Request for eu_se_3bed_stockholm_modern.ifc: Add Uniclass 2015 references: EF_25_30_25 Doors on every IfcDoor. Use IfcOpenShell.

First a look at what the model holds.

```python
import ifcopenshell

model = ifcopenshell.open("eu_se_3bed_stockholm_modern.ifc")
print(model.schema)
print("classifications:", [c.Name for c in model.by_type("IfcClassification")])
for ifc_class in ("IfcDoor", "IfcRoof", "IfcStair", "IfcWall", "IfcWindow"):
    print(ifc_class, len(model.by_type(ifc_class)))
```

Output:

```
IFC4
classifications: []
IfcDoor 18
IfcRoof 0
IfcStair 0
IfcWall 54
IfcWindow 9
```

```python
import ifcopenshell
import ifcopenshell.api.classification

model = ifcopenshell.open("eu_se_3bed_stockholm_modern.ifc")

system = ifcopenshell.api.classification.add_classification(model, classification="Uniclass 2015")

codes = {
    "IfcDoor": ("EF_25_30_25", "Doors"),
}
for ifc_class, (code, name) in codes.items():
    products = model.by_type(ifc_class)
    ifcopenshell.api.classification.add_reference(
        model, products=products, classification=system, identification=code, name=name
    )
    print(code, len(products))

model.write("eu_se_3bed_stockholm_modern_updated.ifc")
```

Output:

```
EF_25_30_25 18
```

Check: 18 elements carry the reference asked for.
